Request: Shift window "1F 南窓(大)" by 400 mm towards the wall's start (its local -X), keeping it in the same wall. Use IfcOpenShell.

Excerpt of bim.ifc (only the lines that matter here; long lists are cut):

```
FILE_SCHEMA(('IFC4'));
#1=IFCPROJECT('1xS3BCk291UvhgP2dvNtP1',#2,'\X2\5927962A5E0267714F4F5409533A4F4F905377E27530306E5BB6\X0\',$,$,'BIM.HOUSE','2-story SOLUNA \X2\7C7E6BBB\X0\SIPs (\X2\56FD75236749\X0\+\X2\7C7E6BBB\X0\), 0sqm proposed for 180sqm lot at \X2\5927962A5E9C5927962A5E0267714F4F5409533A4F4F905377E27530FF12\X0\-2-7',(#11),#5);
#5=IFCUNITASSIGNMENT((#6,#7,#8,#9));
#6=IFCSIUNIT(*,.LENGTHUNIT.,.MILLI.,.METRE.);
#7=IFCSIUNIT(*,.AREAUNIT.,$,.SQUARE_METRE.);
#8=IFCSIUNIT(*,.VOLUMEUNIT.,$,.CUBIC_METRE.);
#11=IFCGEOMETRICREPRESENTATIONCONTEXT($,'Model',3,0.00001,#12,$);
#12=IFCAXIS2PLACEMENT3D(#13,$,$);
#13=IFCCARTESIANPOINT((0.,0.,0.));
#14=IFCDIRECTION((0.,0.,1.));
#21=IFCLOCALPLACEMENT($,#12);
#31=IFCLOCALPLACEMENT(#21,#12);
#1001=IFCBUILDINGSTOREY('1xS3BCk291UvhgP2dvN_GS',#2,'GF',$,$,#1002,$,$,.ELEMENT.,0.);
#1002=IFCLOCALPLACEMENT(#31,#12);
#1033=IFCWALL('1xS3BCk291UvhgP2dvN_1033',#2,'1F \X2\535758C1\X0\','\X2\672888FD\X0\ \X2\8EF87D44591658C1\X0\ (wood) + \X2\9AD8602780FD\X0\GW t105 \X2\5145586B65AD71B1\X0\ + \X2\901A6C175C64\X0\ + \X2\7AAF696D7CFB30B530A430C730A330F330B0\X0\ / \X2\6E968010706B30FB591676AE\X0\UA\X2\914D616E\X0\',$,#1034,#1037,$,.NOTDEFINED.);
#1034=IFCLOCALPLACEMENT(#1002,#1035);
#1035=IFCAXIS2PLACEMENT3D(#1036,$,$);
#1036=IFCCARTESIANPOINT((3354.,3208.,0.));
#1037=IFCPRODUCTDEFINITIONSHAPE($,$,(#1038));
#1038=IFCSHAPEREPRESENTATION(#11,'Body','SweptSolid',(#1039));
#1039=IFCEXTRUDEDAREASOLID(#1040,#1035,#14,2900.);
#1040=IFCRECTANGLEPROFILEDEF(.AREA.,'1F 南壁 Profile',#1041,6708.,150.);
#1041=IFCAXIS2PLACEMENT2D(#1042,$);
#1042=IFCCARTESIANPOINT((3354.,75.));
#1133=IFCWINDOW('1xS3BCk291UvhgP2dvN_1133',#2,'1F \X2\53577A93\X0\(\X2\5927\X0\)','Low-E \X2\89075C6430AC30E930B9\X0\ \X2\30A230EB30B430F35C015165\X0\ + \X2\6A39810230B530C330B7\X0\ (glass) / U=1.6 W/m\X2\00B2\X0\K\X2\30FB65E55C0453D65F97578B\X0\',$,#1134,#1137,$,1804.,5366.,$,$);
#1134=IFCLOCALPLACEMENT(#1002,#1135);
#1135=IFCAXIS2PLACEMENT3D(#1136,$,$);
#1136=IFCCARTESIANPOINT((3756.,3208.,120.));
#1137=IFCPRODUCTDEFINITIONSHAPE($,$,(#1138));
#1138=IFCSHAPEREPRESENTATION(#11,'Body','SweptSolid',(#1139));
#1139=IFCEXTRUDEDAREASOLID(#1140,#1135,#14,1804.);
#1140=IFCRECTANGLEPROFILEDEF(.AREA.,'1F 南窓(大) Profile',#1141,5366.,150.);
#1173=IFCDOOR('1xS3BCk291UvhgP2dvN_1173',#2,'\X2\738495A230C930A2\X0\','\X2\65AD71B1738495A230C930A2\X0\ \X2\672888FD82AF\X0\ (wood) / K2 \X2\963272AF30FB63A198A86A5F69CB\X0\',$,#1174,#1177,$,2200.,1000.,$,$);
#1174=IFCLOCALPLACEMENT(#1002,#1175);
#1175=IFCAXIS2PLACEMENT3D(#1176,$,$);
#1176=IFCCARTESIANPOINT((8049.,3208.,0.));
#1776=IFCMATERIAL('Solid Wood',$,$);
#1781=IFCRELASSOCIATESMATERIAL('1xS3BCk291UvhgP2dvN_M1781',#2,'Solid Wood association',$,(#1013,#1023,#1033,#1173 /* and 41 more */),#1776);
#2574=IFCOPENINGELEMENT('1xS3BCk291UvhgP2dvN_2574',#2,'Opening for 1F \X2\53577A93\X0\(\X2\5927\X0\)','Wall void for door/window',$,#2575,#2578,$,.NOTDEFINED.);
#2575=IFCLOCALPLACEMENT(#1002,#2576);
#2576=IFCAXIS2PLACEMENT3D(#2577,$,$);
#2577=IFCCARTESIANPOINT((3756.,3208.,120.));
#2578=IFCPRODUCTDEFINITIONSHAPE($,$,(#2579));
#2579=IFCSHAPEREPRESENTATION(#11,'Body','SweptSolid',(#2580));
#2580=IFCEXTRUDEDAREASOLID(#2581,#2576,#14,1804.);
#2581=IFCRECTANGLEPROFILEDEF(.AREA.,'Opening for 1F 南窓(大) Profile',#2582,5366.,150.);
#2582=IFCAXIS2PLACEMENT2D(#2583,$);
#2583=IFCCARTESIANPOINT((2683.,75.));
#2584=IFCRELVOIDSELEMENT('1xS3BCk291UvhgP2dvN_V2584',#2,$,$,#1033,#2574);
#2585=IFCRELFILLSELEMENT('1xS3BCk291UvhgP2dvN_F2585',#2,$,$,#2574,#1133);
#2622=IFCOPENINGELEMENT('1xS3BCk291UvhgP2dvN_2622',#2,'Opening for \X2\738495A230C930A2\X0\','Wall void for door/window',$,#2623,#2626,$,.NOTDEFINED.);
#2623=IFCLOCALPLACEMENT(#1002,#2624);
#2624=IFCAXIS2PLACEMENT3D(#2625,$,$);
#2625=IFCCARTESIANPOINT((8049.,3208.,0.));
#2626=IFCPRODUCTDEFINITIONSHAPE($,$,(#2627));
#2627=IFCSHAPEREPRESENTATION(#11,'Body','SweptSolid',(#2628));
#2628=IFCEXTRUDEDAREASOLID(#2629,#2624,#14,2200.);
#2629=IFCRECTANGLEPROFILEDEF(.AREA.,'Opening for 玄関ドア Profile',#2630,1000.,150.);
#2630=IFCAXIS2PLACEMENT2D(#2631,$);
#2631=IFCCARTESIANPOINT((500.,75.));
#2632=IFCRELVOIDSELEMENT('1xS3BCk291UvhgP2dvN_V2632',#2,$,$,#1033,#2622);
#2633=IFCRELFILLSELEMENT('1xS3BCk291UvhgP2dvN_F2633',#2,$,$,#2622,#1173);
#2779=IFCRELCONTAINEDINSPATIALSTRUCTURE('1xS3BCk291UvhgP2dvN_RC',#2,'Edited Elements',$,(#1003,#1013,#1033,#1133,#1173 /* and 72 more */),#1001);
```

```python
import ifcopenshell
import ifcopenshell.api.geometry
import ifcopenshell.util.placement

model = ifcopenshell.open("bim.ifc")

window = model.by_id(1133)
opening = window.FillsVoids[0].RelatingOpeningElement
wall = opening.VoidsElements[0].RelatingBuildingElement

wall_matrix = ifcopenshell.util.placement.get_local_placement(wall.ObjectPlacement)
shift = wall_matrix[:3, 0] * -400.0
before = ifcopenshell.util.placement.get_local_placement(window.ObjectPlacement)[:3, 3].copy()

# The window is not placed relative to its opening, so move both.
for product in (opening, window):
    matrix = ifcopenshell.util.placement.get_local_placement(product.ObjectPlacement)
    matrix[:3, 3] += shift
    ifcopenshell.api.geometry.edit_object_placement(model, product=product, matrix=matrix, is_si=False)

after = ifcopenshell.util.placement.get_local_placement(window.ObjectPlacement)[:3, 3]
print("window moved by", (after - before).round(3) + 0.0)

model.write("bim_edited.ifc")
```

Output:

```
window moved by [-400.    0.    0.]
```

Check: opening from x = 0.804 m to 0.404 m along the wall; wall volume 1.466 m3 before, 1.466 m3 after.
